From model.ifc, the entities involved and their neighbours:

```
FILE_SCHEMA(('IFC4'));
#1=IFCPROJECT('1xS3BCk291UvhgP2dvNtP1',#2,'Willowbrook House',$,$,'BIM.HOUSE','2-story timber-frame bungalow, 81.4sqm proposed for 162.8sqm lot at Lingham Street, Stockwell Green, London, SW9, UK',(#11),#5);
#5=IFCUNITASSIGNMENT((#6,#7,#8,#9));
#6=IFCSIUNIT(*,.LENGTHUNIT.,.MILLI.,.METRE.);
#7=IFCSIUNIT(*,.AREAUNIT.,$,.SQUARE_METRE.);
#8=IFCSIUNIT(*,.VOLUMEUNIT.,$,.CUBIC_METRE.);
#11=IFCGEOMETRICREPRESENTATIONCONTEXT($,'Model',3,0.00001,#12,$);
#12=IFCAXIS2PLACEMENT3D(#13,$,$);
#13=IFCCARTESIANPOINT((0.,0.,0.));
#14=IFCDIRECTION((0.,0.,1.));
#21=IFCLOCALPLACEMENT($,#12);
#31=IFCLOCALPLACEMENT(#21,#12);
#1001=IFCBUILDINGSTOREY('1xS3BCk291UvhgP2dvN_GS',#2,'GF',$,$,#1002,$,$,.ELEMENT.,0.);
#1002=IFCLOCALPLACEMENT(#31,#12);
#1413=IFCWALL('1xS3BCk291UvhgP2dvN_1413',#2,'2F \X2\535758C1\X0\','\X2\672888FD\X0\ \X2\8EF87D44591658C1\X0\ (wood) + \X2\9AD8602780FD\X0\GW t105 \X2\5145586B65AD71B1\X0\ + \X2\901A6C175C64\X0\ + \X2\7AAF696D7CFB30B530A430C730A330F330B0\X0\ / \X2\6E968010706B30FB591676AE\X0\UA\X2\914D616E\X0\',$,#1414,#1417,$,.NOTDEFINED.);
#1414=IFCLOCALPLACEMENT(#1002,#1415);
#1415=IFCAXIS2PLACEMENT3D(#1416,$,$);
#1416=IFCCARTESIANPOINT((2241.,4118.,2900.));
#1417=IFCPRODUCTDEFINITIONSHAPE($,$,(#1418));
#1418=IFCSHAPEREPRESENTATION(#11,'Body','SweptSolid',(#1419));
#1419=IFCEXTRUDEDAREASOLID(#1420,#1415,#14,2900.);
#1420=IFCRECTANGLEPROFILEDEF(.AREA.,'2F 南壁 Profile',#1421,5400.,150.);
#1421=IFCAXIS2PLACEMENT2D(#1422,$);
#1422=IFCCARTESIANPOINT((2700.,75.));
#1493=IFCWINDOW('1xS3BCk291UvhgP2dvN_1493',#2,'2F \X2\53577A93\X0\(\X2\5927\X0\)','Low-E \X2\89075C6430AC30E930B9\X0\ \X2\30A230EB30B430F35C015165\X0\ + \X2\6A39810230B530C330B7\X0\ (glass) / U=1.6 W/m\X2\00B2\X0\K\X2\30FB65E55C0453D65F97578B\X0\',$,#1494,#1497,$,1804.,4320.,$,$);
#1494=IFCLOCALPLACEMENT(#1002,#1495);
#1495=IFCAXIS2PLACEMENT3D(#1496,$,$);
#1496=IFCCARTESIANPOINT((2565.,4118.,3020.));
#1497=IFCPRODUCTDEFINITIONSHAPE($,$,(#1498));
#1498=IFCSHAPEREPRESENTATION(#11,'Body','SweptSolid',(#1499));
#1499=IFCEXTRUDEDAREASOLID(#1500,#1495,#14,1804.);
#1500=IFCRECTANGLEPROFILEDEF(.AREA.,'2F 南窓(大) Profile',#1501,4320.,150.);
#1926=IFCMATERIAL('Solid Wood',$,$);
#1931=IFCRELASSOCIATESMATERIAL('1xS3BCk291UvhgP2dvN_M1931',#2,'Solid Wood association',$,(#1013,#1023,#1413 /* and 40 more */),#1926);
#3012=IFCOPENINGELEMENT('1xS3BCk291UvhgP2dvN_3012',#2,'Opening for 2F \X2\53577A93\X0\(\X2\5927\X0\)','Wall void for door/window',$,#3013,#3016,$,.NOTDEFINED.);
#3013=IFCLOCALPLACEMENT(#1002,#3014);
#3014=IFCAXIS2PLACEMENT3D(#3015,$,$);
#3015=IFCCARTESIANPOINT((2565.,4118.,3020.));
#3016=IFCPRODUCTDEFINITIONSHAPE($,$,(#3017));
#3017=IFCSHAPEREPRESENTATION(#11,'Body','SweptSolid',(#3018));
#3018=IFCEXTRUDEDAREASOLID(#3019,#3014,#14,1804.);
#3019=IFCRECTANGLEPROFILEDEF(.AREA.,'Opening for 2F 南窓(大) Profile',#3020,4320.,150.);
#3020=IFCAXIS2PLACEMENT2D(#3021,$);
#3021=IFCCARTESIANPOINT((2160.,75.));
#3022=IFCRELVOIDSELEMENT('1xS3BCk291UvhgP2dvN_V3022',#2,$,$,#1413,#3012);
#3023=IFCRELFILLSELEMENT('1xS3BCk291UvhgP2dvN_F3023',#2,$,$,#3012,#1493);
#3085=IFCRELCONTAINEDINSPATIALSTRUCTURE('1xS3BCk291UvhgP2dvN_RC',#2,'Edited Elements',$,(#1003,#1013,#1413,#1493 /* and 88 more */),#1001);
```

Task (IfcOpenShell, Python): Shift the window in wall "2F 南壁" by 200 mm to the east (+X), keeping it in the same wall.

```python
import ifcopenshell
import ifcopenshell.api.geometry
import ifcopenshell.util.placement
import ifcopenshell.util.unit

model = ifcopenshell.open("model.ifc")
unit_scale = ifcopenshell.util.unit.calculate_unit_scale(model)

window = model.by_id(1493)
opening = window.FillsVoids[0].RelatingOpeningElement
wall = opening.VoidsElements[0].RelatingBuildingElement

wall_matrix = ifcopenshell.util.placement.get_local_placement(wall.ObjectPlacement)
shift = wall_matrix[:3, 0] * 0.2 / unit_scale
before = ifcopenshell.util.placement.get_local_placement(window.ObjectPlacement)[:3, 3].copy()

# The window is not placed relative to its opening, so move both.
for product in (opening, window):
    matrix = ifcopenshell.util.placement.get_local_placement(product.ObjectPlacement)
    matrix[:3, 3] += shift
    ifcopenshell.api.geometry.edit_object_placement(model, product=product, matrix=matrix, is_si=False)

after = ifcopenshell.util.placement.get_local_placement(window.ObjectPlacement)[:3, 3]
print("window moved by", (after - before).round(3) + 0.0)

model.write("model_updated.ifc")
```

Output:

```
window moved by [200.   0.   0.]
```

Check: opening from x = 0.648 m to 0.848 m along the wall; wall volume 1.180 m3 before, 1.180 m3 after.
